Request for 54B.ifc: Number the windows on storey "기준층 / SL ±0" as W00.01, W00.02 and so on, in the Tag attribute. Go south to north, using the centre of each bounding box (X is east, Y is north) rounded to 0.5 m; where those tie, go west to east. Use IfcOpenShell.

First a look at what the model holds.

```python
import ifcopenshell
import ifcopenshell.util.element
import ifcopenshell.util.placement

model = ifcopenshell.open("54B.ifc")
print(model.schema)
storey = next(s for s in model.by_type("IfcBuildingStorey") if s.Name == "기준층 / SL ±0")
windows = [e for e in ifcopenshell.util.element.get_decomposition(storey) if e.is_a("IfcWindow")]
for e in sorted(windows, key=lambda e: e.id()):
    origin = ifcopenshell.util.placement.get_local_placement(e.ObjectPlacement)[:3, 3]
    print(e.id(), e.Tag, e.Name, origin.round(2) + 0.0, sep=" | ")
```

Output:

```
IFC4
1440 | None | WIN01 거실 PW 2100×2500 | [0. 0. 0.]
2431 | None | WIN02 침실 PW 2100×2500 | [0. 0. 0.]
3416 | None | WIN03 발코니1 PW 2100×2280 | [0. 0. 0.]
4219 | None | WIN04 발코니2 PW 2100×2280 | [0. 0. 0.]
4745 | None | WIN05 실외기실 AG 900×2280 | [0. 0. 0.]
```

```python
import ifcopenshell
import ifcopenshell.geom
import ifcopenshell.util.element
import ifcopenshell.util.shape

model = ifcopenshell.open("54B.ifc")
settings = ifcopenshell.geom.settings()
settings.set("use-world-coords", True)


def centre(element):
    shape = ifcopenshell.geom.create_shape(settings, element)
    return ifcopenshell.util.shape.get_bbox_centroid(shape.geometry)


storey = next(s for s in model.by_type("IfcBuildingStorey") if s.Name == "기준층 / SL ±0")
windows = [e for e in ifcopenshell.util.element.get_decomposition(storey) if e.is_a("IfcWindow")]

# Insertion points can sit at a corner or the storey origin, so sort by the geometry (in metres).
centres = {e: centre(e) for e in windows}
windows.sort(key=lambda e: (round(centres[e][1] / 0.5), centres[e][0]))

for i, e in enumerate(windows, start=1):
    number = f"W00.{i:02d}"
    e.Tag = number
    print(e.id(), number)

model.write("54B_edited.ifc")
```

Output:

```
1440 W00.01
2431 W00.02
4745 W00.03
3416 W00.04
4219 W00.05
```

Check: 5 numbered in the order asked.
